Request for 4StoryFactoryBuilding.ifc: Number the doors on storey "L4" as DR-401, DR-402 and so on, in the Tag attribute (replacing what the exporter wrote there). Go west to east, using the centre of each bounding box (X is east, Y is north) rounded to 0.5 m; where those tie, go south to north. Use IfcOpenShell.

First a look at what the model holds.

```python
import ifcopenshell
import ifcopenshell.util.element
import ifcopenshell.util.placement

model = ifcopenshell.open("4StoryFactoryBuilding.ifc")
print(model.schema)
storey = next(s for s in model.by_type("IfcBuildingStorey") if s.Name == "L4")
doors = [e for e in ifcopenshell.util.element.get_decomposition(storey) if e.is_a("IfcDoor")]
for e in sorted(doors, key=lambda e: e.id()):
    origin = ifcopenshell.util.placement.get_local_placement(e.ObjectPlacement)[:3, 3]
    print(e.id(), e.Tag, e.Name, origin.round(2) + 0.0, sep=" | ")
```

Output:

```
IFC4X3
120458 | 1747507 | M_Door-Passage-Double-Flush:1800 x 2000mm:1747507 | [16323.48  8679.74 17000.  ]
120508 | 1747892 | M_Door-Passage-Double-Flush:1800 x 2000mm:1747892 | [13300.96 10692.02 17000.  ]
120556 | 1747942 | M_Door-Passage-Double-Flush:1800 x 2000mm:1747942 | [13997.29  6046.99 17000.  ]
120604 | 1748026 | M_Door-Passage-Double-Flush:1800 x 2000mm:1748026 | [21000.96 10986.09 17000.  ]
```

```python
import ifcopenshell
import ifcopenshell.geom
import ifcopenshell.util.element
import ifcopenshell.util.shape

model = ifcopenshell.open("4StoryFactoryBuilding.ifc")
settings = ifcopenshell.geom.settings()
settings.set("use-world-coords", True)


def centre(element):
    shape = ifcopenshell.geom.create_shape(settings, element)
    return ifcopenshell.util.shape.get_bbox_centroid(shape.geometry)


storey = next(s for s in model.by_type("IfcBuildingStorey") if s.Name == "L4")
doors = [e for e in ifcopenshell.util.element.get_decomposition(storey) if e.is_a("IfcDoor")]

# Insertion points can sit at a corner or the storey origin, so sort by the geometry (in metres).
centres = {e: centre(e) for e in doors}
doors.sort(key=lambda e: (round(centres[e][0] / 0.5), centres[e][1]))

for i, e in enumerate(doors, start=1):
    number = f"DR-4{i:02d}"
    e.Tag = number
    print(e.id(), number)

model.write("4StoryFactoryBuilding_updated.ifc")
```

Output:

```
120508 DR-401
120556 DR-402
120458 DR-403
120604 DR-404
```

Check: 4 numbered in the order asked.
